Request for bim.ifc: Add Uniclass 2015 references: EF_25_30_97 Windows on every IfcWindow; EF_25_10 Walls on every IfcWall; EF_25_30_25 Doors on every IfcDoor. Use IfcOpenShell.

First a look at what the model holds.

```python
import ifcopenshell

model = ifcopenshell.open("bim.ifc")
print(model.schema)
print("classifications:", [c.Name for c in model.by_type("IfcClassification")])
for ifc_class in ("IfcDoor", "IfcRoof", "IfcStair", "IfcWall", "IfcWindow"):
    print(ifc_class, len(model.by_type(ifc_class)))
```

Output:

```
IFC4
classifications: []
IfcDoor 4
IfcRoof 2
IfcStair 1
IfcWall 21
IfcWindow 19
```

```python
import ifcopenshell
import ifcopenshell.api.classification

model = ifcopenshell.open("bim.ifc")

system = ifcopenshell.api.classification.add_classification(model, classification="Uniclass 2015")

codes = {
    "IfcWindow": ("EF_25_30_97", "Windows"),
    "IfcWall": ("EF_25_10", "Walls"),
    "IfcDoor": ("EF_25_30_25", "Doors"),
}
for ifc_class, (code, name) in codes.items():
    products = model.by_type(ifc_class)
    ifcopenshell.api.classification.add_reference(
        model, products=products, classification=system, identification=code, name=name
    )
    print(code, len(products))

model.write("bim_updated.ifc")
```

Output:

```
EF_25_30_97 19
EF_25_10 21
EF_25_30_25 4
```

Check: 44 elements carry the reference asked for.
